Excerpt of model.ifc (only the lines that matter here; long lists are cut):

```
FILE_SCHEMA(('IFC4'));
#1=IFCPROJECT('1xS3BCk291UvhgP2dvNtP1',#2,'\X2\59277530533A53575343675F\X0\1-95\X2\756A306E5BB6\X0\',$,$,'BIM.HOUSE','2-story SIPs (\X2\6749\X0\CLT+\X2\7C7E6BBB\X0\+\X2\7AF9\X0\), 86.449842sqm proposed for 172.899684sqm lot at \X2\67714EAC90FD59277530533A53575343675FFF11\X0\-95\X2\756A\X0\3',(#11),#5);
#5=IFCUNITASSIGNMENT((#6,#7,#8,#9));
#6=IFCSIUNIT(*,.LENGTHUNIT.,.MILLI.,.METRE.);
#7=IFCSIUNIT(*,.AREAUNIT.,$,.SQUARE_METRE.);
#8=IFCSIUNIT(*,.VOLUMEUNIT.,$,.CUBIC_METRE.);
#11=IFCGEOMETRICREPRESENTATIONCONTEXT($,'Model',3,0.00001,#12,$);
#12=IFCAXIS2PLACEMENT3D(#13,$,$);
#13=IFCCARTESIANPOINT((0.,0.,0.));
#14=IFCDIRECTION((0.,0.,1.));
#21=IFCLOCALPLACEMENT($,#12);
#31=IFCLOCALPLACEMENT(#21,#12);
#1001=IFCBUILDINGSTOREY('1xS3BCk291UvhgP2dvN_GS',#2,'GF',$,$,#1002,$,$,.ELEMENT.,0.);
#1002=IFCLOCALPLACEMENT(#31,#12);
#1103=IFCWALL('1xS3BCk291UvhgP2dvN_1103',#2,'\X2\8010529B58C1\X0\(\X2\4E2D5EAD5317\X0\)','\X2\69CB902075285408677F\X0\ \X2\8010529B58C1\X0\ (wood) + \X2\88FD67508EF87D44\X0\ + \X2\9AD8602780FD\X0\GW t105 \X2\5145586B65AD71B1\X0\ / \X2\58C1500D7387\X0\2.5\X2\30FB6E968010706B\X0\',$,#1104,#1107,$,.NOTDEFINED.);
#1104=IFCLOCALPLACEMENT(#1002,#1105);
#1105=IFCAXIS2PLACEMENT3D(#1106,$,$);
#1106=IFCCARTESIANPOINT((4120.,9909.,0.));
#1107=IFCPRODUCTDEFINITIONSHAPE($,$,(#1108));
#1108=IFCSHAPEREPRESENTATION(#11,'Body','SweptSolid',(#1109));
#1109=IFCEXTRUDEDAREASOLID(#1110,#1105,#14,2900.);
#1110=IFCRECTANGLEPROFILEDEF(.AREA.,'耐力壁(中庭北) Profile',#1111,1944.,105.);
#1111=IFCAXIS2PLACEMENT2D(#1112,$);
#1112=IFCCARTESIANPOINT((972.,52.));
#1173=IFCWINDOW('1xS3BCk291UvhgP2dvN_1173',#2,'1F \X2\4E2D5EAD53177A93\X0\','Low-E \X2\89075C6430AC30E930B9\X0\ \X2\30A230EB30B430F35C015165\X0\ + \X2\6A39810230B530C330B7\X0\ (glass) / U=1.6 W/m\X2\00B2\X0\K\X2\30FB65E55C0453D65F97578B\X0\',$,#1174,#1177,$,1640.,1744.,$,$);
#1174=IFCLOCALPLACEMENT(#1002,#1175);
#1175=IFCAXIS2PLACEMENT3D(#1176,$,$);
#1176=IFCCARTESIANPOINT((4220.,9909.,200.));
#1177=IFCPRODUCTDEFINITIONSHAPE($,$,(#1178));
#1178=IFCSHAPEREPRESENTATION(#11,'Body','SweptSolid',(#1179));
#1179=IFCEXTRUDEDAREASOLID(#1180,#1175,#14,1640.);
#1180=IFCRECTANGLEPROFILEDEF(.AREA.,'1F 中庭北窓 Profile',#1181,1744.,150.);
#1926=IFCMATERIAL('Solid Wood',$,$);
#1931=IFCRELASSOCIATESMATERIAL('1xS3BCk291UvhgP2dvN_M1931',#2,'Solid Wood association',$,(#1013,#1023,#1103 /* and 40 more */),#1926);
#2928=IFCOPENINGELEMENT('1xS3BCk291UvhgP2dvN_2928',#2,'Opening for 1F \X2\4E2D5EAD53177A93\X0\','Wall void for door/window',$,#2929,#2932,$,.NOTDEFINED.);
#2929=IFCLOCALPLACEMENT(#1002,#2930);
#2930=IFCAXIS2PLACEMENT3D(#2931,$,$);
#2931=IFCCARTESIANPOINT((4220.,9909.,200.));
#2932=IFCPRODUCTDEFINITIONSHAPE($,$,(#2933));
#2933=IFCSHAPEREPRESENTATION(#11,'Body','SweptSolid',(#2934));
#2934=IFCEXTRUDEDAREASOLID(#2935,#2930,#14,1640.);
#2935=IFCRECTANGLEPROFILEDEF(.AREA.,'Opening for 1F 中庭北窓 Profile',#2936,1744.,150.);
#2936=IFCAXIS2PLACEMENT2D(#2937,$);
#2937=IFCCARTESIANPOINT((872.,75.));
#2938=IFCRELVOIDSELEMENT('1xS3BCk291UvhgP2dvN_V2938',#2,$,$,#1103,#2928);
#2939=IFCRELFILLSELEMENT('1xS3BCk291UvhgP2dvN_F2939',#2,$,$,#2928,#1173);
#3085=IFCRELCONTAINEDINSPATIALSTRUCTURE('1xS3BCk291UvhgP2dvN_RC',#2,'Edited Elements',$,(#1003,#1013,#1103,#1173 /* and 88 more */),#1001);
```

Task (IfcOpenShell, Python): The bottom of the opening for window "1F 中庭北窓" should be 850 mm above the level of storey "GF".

```python
import numpy as np
import ifcopenshell
import ifcopenshell.api.geometry
import ifcopenshell.geom
import ifcopenshell.util.element
import ifcopenshell.util.placement
import ifcopenshell.util.shape
import ifcopenshell.util.unit

model = ifcopenshell.open("model.ifc")
unit_scale = ifcopenshell.util.unit.calculate_unit_scale(model)

window = model.by_id(1173)
opening = window.FillsVoids[0].RelatingOpeningElement
storey = ifcopenshell.util.element.get_container(window, ifc_class="IfcBuildingStorey")
level = ifcopenshell.util.placement.get_local_placement(storey.ObjectPlacement)[2, 3]

# The opening's origin need not be at the sill, so measure its lowest point.
shape = ifcopenshell.geom.create_shape(ifcopenshell.geom.settings(), opening)
bottom = ifcopenshell.util.shape.get_shape_bottom_elevation(shape, shape.geometry) / unit_scale
dz = level + 0.85 / unit_scale - bottom

shift = np.array([0.0, 0.0, dz])
# The window is not placed relative to its opening, so move both.
for product in (opening, window):
    matrix = ifcopenshell.util.placement.get_local_placement(product.ObjectPlacement)
    matrix[:3, 3] += shift
    ifcopenshell.api.geometry.edit_object_placement(model, product=product, matrix=matrix, is_si=False)

print(f"moved by {dz * unit_scale:+.3f} m")

model.write("model_updated.ifc")
```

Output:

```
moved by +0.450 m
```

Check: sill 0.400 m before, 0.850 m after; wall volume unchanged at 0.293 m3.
